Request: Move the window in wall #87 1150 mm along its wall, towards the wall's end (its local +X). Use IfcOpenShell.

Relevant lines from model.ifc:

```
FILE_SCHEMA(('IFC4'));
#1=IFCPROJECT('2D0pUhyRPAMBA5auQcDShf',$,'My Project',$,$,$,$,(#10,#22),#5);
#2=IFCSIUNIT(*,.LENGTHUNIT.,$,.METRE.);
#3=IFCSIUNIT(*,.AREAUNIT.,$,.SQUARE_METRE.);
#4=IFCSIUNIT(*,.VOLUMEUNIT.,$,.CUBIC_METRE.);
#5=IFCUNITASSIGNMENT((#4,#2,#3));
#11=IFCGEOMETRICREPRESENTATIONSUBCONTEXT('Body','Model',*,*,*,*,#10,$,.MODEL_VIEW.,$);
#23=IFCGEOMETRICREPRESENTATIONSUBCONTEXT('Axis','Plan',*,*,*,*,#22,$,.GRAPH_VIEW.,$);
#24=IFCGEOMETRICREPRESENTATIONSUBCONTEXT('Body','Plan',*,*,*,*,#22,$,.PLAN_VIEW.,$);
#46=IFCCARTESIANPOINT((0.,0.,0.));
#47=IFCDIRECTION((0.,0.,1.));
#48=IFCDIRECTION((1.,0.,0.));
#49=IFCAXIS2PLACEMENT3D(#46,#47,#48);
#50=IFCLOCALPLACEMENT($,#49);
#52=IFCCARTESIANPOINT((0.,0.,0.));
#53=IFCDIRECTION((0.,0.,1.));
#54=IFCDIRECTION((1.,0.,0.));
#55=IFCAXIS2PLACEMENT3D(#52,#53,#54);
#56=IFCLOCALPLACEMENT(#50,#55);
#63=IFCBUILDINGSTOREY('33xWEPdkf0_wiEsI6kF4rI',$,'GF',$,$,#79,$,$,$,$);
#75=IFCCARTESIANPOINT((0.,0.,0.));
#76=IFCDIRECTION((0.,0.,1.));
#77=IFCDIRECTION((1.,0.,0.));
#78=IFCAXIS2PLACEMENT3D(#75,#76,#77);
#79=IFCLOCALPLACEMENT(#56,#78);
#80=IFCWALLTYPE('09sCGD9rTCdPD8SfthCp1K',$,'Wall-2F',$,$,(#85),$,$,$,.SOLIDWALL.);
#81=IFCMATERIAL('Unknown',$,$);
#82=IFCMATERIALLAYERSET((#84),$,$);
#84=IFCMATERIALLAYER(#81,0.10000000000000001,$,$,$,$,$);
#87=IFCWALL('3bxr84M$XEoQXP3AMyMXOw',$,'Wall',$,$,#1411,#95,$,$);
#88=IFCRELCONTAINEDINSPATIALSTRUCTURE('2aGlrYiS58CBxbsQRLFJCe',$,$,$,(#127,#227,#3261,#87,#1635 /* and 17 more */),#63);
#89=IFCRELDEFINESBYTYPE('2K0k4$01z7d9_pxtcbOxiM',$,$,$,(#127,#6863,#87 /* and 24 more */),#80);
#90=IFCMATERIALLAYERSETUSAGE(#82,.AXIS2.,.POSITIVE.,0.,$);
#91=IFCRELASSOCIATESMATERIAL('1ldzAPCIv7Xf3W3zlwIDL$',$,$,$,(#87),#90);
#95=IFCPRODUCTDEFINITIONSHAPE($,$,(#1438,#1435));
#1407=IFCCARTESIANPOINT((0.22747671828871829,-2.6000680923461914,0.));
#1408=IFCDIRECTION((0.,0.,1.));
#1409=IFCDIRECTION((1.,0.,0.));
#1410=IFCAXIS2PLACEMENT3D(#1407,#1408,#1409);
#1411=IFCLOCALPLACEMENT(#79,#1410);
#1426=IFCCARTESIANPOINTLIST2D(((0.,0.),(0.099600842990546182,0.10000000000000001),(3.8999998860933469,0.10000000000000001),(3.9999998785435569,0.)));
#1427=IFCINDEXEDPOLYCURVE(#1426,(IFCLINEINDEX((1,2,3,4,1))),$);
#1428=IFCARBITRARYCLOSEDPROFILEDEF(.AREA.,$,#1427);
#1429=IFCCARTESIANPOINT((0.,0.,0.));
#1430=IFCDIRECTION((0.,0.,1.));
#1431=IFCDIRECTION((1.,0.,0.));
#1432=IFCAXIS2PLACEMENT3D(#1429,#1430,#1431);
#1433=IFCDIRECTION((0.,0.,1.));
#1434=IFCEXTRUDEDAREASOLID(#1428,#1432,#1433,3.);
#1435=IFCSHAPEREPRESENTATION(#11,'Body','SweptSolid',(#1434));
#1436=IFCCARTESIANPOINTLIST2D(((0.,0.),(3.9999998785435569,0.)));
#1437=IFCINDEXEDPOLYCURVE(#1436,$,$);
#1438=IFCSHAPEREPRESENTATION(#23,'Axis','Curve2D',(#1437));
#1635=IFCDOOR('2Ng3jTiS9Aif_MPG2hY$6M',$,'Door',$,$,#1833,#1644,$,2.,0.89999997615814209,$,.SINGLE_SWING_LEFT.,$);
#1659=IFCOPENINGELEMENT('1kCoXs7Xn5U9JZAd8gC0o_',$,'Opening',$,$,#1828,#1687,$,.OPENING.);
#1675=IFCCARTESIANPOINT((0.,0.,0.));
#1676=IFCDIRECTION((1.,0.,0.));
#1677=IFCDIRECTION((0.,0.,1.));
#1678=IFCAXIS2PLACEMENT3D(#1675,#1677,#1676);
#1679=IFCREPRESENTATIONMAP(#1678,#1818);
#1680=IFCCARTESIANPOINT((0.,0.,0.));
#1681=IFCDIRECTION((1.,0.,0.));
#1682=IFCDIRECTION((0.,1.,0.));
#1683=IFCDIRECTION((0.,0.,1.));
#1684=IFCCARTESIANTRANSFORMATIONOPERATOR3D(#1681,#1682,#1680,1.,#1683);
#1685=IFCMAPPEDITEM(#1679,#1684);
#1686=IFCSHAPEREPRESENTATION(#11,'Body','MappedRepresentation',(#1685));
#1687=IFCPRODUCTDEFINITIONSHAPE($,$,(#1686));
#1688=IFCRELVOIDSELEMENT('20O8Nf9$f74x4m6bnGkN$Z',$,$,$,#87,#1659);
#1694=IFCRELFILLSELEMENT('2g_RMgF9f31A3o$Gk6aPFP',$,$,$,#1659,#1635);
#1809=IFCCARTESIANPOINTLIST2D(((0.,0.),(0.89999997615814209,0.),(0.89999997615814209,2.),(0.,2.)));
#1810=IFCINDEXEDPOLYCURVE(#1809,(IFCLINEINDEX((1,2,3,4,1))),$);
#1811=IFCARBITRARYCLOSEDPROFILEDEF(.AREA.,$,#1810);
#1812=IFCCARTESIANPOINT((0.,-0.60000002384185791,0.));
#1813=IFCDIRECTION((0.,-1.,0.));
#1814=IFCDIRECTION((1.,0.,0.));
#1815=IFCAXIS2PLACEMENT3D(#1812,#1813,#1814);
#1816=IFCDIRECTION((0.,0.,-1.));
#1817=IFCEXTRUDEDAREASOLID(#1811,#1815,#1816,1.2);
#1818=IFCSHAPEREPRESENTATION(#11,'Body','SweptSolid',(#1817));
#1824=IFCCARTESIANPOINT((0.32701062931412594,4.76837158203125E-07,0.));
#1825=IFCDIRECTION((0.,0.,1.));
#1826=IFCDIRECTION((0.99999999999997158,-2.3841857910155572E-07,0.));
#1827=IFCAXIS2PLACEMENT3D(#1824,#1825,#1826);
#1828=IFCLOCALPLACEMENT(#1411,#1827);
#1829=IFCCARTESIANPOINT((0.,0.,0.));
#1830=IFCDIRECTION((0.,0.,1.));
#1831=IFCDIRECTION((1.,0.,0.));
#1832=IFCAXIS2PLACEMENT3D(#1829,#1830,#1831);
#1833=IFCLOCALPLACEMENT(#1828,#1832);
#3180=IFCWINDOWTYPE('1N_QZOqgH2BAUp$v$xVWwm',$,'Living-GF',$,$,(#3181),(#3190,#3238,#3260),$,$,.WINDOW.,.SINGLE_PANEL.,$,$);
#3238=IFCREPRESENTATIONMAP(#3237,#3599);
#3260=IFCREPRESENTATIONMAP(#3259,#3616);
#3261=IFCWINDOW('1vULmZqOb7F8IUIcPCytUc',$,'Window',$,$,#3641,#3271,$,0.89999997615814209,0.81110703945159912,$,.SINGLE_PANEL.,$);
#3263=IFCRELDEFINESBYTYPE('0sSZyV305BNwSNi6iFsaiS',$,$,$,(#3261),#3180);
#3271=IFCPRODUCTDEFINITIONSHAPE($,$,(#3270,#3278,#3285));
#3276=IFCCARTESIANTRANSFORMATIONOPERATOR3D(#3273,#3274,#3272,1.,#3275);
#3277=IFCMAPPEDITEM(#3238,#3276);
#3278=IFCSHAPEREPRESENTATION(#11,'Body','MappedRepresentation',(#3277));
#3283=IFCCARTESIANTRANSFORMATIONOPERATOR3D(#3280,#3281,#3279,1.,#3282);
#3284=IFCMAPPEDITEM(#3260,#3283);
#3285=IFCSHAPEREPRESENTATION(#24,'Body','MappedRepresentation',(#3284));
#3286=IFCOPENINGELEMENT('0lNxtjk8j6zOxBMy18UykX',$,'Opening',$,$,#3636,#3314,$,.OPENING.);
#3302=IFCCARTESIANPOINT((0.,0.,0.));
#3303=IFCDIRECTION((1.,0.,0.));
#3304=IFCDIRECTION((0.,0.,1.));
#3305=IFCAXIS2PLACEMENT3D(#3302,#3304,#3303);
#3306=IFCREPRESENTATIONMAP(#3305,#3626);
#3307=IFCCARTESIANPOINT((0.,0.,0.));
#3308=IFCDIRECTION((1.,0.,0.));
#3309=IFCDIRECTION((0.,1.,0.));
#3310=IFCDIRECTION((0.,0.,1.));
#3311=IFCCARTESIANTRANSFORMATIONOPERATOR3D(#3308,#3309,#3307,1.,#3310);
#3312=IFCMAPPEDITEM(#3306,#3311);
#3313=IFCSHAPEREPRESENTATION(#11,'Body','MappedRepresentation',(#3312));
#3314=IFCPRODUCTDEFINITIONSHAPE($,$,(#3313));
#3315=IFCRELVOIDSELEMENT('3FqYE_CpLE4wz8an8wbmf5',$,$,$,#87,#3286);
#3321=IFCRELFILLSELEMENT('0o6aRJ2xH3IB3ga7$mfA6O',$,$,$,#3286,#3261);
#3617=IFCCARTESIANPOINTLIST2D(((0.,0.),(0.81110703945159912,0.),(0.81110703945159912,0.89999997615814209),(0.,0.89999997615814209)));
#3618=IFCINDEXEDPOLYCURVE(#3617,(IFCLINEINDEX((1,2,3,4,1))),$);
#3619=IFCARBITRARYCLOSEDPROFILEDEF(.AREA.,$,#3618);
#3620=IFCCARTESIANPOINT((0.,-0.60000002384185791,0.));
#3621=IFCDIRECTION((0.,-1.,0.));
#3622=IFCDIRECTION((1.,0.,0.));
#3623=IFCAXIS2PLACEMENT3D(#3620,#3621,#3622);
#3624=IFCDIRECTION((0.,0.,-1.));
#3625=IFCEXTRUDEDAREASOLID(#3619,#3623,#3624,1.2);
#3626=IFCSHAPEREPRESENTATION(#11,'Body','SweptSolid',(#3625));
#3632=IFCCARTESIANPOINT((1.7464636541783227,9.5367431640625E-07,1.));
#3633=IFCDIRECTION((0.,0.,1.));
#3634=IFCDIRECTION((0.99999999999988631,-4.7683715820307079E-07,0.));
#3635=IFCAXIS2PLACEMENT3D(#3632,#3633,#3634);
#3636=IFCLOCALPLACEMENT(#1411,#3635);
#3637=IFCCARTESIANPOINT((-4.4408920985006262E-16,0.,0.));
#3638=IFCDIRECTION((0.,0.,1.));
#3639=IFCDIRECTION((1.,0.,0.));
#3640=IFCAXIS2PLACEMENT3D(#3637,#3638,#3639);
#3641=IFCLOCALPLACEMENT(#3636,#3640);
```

```python
import ifcopenshell
import ifcopenshell.api.geometry
import ifcopenshell.util.placement
import ifcopenshell.util.unit

model = ifcopenshell.open("model.ifc")
unit_scale = ifcopenshell.util.unit.calculate_unit_scale(model)

window = model.by_id(3261)
opening = window.FillsVoids[0].RelatingOpeningElement
wall = opening.VoidsElements[0].RelatingBuildingElement

wall_matrix = ifcopenshell.util.placement.get_local_placement(wall.ObjectPlacement)
shift = wall_matrix[:3, 0] * 1.15 / unit_scale
before = ifcopenshell.util.placement.get_local_placement(window.ObjectPlacement)[:3, 3].copy()

# The window is placed relative to its opening, so it follows when the opening moves.
matrix = ifcopenshell.util.placement.get_local_placement(opening.ObjectPlacement)
matrix[:3, 3] += shift
ifcopenshell.api.geometry.edit_object_placement(
    model, product=opening, matrix=matrix, is_si=False, should_transform_children=True
)

after = ifcopenshell.util.placement.get_local_placement(window.ObjectPlacement)[:3, 3]
print("window moved by", (after - before).round(3) + 0.0)

model.write("model-out.ifc")
```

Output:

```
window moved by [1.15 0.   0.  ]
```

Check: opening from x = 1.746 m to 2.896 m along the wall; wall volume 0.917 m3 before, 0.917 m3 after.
